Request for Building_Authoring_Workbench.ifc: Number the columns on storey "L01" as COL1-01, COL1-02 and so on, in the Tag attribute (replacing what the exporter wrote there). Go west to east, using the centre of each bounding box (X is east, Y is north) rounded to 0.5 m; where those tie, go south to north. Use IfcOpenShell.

First a look at what the model holds.

```python
import ifcopenshell
import ifcopenshell.util.element
import ifcopenshell.util.placement

model = ifcopenshell.open("Building_Authoring_Workbench.ifc")
print(model.schema)
storey = next(s for s in model.by_type("IfcBuildingStorey") if s.Name == "L01")
columns = [e for e in ifcopenshell.util.element.get_decomposition(storey) if e.is_a("IfcColumn")]
for e in sorted(columns, key=lambda e: e.id()):
    origin = ifcopenshell.util.placement.get_local_placement(e.ObjectPlacement)[:3, 3]
    print(e.id(), e.Tag, e.Name, origin.round(2) + 0.0, sep=" | ")
```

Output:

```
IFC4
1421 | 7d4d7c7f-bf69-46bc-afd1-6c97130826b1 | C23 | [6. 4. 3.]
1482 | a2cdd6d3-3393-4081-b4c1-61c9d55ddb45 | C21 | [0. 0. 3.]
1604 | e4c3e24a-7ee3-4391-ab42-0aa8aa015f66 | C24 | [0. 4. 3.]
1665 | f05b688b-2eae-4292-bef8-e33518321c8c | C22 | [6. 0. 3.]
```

```python
import ifcopenshell
import ifcopenshell.geom
import ifcopenshell.util.element
import ifcopenshell.util.shape

model = ifcopenshell.open("Building_Authoring_Workbench.ifc")
settings = ifcopenshell.geom.settings()
settings.set("use-world-coords", True)


def centre(element):
    shape = ifcopenshell.geom.create_shape(settings, element)
    return ifcopenshell.util.shape.get_bbox_centroid(shape.geometry)


storey = next(s for s in model.by_type("IfcBuildingStorey") if s.Name == "L01")
columns = [e for e in ifcopenshell.util.element.get_decomposition(storey) if e.is_a("IfcColumn")]

# Insertion points can sit at a corner or the storey origin, so sort by the geometry (in metres).
centres = {e: centre(e) for e in columns}
columns.sort(key=lambda e: (round(centres[e][0] / 0.5), centres[e][1]))

for i, e in enumerate(columns, start=1):
    number = f"COL1-{i:02d}"
    e.Tag = number
    print(e.id(), number)

model.write("Building_Authoring_Workbench-out.ifc")
```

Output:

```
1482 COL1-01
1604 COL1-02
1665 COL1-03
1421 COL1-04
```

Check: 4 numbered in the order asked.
